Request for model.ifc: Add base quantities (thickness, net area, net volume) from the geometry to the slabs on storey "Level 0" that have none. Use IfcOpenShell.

First a look at what the model holds.

```python
import ifcopenshell
import ifcopenshell.util.element
import ifcopenshell.util.unit

model = ifcopenshell.open("model.ifc")
print(model.schema)
for unit_type in ("LENGTHUNIT", "AREAUNIT", "VOLUMEUNIT"):
    print(unit_type, ifcopenshell.util.unit.calculate_unit_scale(model, unit_type))
storey = next(s for s in model.by_type("IfcBuildingStorey") if s.Name == "Level 0")
slabs = [e for e in ifcopenshell.util.element.get_decomposition(storey) if e.is_a("IfcSlab")]
for e in sorted(slabs, key=lambda e: e.id()):
    print(e.id(), e.is_a(), e.Name, list(ifcopenshell.util.element.get_psets(e, qtos_only=True)), sep=" | ")
```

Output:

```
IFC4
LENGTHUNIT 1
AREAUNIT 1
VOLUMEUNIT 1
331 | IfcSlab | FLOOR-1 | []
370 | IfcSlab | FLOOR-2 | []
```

```python
import ifcopenshell
import ifcopenshell.api.pset
import ifcopenshell.geom
import ifcopenshell.util.element
import ifcopenshell.util.shape
import ifcopenshell.util.unit

model = ifcopenshell.open("model.ifc")
unit_scale = ifcopenshell.util.unit.calculate_unit_scale(model)
area_scale = ifcopenshell.util.unit.calculate_unit_scale(model, "AREAUNIT")
volume_scale = ifcopenshell.util.unit.calculate_unit_scale(model, "VOLUMEUNIT")
settings = ifcopenshell.geom.settings()

storey = next(s for s in model.by_type("IfcBuildingStorey") if s.Name == "Level 0")
slabs = [e for e in ifcopenshell.util.element.get_decomposition(storey) if e.is_a("IfcSlab")]

for e in sorted(slabs, key=lambda e: e.id()):
    if ifcopenshell.util.element.get_psets(e, qtos_only=True, should_inherit=False):
        continue
    # Geometry comes back in metres, in the element's own axes.
    shape = ifcopenshell.geom.create_shape(settings, e)
    values = {
        "Width": ifcopenshell.util.shape.get_z(shape.geometry) / unit_scale,
        "NetArea": ifcopenshell.util.shape.get_footprint_area(shape.geometry) / area_scale,
        "NetVolume": ifcopenshell.util.shape.get_volume(shape.geometry) / volume_scale,
    }
    qto = ifcopenshell.api.pset.add_qto(model, product=e, name="Qto_SlabBaseQuantities")
    ifcopenshell.api.pset.edit_qto(model, qto=qto, properties=values)
    print(e.id(), {k: round(v, 3) for k, v in values.items()})

model.write("model_updated.ifc")
```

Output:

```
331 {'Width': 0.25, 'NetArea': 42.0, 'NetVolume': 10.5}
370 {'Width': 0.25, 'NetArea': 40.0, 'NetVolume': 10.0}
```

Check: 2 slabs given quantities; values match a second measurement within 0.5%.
